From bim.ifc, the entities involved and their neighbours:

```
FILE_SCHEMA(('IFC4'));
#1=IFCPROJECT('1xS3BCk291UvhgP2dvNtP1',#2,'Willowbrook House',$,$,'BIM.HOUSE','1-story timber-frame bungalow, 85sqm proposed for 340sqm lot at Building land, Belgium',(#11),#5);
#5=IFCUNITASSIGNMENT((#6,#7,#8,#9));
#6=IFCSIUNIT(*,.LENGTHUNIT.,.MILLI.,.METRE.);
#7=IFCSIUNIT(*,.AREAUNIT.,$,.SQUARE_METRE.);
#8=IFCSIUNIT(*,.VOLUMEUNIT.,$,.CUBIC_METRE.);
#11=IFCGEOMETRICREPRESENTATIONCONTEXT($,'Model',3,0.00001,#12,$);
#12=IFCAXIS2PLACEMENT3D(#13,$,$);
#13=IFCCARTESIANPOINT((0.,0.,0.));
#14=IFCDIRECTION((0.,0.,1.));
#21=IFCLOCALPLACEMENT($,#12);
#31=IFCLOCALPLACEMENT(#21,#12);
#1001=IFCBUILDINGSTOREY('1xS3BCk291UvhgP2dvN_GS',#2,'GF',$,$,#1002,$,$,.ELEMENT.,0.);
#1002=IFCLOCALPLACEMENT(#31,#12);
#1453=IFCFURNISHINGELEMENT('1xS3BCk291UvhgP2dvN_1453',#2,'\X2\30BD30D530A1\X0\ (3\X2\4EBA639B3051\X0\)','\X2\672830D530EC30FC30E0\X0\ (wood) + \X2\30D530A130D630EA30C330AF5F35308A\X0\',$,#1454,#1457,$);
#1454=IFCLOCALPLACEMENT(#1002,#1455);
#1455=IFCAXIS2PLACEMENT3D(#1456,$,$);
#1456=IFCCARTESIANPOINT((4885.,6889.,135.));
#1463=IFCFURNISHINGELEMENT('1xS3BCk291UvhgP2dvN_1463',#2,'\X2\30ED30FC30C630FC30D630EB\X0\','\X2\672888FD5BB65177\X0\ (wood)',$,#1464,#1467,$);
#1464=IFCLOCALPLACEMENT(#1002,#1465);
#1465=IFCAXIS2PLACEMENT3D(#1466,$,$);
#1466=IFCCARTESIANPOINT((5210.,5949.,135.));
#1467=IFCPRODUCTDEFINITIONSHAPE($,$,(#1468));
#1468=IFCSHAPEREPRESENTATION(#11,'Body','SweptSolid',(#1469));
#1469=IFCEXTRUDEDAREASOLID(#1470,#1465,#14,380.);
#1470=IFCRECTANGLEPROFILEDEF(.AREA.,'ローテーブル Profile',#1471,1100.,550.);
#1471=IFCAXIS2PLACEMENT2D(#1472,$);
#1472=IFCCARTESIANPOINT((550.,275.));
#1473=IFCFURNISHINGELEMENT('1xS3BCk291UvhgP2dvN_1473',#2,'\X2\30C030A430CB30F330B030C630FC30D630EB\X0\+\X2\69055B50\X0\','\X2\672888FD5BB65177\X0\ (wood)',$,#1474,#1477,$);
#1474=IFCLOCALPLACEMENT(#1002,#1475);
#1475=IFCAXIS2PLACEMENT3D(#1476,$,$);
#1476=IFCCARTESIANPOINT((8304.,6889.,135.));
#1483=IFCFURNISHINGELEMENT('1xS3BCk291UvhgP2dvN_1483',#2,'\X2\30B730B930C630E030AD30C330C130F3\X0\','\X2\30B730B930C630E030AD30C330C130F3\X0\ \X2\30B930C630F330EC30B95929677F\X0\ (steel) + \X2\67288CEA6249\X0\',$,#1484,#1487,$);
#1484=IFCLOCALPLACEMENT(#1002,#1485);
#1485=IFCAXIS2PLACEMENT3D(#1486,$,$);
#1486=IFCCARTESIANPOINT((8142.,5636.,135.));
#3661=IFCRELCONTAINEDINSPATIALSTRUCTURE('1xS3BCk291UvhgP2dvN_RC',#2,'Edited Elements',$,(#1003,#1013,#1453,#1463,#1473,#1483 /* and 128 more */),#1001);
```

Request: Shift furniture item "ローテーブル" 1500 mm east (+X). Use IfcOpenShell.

```python
import ifcopenshell
import ifcopenshell.api.geometry
import ifcopenshell.util.placement
import ifcopenshell.util.unit

model = ifcopenshell.open("bim.ifc")
unit_scale = ifcopenshell.util.unit.calculate_unit_scale(model)

item = model.by_guid("1xS3BCk291UvhgP2dvN_1463")
matrix = ifcopenshell.util.placement.get_local_placement(item.ObjectPlacement)
matrix[0, 3] += 1.5 / unit_scale
ifcopenshell.api.geometry.edit_object_placement(model, product=item, matrix=matrix, is_si=False)

print(ifcopenshell.util.placement.get_local_placement(item.ObjectPlacement).round(3) + 0.0)

model.write("bim_rev.ifc")
```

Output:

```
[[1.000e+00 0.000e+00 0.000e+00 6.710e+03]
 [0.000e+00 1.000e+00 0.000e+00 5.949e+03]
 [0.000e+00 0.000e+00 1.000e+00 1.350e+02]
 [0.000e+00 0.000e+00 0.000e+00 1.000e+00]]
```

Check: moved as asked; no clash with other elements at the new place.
